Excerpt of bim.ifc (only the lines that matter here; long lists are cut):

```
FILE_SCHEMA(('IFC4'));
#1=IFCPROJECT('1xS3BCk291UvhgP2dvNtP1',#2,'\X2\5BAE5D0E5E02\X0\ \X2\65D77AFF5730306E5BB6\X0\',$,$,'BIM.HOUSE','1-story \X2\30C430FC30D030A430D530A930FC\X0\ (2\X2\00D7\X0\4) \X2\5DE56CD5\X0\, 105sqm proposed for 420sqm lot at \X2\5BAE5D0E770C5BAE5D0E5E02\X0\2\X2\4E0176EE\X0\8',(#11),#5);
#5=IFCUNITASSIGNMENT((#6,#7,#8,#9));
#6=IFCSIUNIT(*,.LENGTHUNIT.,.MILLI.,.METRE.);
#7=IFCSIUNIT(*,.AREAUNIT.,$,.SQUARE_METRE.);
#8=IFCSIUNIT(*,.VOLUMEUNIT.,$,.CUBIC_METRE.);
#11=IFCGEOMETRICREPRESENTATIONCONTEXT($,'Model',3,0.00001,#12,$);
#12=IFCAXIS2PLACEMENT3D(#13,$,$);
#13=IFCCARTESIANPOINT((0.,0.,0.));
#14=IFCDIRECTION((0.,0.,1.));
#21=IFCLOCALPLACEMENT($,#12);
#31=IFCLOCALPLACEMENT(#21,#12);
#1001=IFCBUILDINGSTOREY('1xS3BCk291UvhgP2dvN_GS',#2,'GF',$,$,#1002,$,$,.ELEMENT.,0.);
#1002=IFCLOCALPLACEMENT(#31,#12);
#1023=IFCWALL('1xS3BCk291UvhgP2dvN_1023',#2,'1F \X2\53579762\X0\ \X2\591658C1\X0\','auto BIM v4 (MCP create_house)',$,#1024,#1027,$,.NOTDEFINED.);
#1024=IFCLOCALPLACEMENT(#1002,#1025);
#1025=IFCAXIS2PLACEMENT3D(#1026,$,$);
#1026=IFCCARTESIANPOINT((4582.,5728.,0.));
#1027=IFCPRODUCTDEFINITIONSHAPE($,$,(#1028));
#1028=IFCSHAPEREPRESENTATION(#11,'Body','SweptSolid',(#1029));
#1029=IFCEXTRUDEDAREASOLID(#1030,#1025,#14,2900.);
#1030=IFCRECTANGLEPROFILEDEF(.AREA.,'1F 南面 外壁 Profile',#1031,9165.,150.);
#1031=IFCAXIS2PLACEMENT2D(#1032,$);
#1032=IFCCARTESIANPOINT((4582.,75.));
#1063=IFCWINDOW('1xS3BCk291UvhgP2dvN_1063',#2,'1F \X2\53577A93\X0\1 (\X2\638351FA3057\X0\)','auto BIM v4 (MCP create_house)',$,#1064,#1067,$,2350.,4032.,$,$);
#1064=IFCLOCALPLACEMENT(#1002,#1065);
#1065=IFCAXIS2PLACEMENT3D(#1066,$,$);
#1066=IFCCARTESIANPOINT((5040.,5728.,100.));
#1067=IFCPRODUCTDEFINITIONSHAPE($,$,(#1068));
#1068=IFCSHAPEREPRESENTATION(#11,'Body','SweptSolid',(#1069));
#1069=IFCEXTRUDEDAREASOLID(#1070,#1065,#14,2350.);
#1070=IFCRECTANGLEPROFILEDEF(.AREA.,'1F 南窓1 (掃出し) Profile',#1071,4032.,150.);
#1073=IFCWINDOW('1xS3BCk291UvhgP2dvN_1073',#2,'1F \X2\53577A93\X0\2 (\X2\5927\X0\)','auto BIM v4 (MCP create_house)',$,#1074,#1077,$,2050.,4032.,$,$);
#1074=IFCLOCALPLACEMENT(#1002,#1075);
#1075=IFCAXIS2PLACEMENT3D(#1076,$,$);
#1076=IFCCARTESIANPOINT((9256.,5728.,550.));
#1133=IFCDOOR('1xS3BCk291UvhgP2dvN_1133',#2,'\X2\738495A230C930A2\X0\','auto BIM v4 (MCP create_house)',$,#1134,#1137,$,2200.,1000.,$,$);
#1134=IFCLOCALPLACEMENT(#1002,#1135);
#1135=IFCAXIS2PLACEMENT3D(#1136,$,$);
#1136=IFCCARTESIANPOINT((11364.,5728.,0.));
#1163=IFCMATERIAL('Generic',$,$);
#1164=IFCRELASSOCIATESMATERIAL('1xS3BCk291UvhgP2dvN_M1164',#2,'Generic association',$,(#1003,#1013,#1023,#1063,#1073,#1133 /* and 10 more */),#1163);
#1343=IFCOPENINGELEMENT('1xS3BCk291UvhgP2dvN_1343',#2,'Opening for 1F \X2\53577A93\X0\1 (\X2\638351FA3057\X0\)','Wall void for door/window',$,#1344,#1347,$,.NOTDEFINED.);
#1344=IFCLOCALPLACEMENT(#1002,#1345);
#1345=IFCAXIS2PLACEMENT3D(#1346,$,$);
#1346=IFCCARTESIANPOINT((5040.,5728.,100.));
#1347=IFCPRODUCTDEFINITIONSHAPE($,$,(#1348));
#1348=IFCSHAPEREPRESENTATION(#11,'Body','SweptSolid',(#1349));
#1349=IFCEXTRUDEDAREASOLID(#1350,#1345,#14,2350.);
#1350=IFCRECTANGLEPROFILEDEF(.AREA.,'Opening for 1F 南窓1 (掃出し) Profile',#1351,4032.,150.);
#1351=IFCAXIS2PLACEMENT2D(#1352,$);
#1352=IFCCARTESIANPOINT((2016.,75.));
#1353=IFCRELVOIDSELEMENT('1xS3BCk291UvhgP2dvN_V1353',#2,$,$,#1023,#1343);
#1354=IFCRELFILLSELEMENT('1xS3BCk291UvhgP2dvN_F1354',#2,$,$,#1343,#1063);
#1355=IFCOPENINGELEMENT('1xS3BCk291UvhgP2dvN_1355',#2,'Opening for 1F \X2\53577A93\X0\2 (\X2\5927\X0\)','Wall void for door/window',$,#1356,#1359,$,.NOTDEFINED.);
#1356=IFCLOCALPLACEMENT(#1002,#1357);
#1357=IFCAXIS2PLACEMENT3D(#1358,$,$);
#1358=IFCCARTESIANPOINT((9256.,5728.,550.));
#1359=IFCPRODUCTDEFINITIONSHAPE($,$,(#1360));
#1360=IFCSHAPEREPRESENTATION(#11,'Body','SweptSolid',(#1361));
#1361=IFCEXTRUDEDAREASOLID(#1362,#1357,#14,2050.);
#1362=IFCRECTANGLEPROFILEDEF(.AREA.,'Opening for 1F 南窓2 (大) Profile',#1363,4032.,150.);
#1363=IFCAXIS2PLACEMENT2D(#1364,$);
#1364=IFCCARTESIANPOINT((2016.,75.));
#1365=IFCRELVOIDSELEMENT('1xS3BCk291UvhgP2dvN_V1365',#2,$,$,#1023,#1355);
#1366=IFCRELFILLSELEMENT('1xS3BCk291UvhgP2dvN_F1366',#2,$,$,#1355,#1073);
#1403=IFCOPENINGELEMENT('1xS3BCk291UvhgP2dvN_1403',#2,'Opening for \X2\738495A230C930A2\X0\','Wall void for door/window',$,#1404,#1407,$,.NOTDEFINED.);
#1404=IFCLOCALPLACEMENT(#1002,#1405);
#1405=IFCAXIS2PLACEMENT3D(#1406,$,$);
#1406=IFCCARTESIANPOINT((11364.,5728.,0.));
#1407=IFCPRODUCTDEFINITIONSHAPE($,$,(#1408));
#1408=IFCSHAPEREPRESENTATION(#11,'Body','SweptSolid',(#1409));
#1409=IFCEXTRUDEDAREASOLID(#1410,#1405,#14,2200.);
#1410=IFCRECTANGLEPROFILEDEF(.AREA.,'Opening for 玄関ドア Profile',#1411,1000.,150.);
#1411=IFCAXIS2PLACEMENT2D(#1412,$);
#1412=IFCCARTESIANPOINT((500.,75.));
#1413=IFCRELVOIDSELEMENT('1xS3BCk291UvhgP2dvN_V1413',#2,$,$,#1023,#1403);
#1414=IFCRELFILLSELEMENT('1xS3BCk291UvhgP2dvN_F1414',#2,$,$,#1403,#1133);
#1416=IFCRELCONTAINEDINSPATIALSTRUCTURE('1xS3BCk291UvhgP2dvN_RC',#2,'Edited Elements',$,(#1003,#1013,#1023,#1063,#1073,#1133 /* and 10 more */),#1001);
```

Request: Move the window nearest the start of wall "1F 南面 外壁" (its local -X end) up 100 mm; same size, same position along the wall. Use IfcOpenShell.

```python
import numpy as np
import ifcopenshell
import ifcopenshell.api.geometry
import ifcopenshell.util.placement
import ifcopenshell.util.unit

model = ifcopenshell.open("bim.ifc")
unit_scale = ifcopenshell.util.unit.calculate_unit_scale(model)

window = model.by_guid("1xS3BCk291UvhgP2dvN_1063")
opening = window.FillsVoids[0].RelatingOpeningElement
dz = 100.0

shift = np.array([0.0, 0.0, dz])
# The window is not placed relative to its opening, so move both.
for product in (opening, window):
    matrix = ifcopenshell.util.placement.get_local_placement(product.ObjectPlacement)
    matrix[:3, 3] += shift
    ifcopenshell.api.geometry.edit_object_placement(model, product=product, matrix=matrix, is_si=False)

print(f"moved by {dz * unit_scale:+.3f} m")

model.write("bim_v2.ifc")
```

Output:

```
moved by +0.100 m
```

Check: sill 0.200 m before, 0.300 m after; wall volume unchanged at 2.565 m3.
